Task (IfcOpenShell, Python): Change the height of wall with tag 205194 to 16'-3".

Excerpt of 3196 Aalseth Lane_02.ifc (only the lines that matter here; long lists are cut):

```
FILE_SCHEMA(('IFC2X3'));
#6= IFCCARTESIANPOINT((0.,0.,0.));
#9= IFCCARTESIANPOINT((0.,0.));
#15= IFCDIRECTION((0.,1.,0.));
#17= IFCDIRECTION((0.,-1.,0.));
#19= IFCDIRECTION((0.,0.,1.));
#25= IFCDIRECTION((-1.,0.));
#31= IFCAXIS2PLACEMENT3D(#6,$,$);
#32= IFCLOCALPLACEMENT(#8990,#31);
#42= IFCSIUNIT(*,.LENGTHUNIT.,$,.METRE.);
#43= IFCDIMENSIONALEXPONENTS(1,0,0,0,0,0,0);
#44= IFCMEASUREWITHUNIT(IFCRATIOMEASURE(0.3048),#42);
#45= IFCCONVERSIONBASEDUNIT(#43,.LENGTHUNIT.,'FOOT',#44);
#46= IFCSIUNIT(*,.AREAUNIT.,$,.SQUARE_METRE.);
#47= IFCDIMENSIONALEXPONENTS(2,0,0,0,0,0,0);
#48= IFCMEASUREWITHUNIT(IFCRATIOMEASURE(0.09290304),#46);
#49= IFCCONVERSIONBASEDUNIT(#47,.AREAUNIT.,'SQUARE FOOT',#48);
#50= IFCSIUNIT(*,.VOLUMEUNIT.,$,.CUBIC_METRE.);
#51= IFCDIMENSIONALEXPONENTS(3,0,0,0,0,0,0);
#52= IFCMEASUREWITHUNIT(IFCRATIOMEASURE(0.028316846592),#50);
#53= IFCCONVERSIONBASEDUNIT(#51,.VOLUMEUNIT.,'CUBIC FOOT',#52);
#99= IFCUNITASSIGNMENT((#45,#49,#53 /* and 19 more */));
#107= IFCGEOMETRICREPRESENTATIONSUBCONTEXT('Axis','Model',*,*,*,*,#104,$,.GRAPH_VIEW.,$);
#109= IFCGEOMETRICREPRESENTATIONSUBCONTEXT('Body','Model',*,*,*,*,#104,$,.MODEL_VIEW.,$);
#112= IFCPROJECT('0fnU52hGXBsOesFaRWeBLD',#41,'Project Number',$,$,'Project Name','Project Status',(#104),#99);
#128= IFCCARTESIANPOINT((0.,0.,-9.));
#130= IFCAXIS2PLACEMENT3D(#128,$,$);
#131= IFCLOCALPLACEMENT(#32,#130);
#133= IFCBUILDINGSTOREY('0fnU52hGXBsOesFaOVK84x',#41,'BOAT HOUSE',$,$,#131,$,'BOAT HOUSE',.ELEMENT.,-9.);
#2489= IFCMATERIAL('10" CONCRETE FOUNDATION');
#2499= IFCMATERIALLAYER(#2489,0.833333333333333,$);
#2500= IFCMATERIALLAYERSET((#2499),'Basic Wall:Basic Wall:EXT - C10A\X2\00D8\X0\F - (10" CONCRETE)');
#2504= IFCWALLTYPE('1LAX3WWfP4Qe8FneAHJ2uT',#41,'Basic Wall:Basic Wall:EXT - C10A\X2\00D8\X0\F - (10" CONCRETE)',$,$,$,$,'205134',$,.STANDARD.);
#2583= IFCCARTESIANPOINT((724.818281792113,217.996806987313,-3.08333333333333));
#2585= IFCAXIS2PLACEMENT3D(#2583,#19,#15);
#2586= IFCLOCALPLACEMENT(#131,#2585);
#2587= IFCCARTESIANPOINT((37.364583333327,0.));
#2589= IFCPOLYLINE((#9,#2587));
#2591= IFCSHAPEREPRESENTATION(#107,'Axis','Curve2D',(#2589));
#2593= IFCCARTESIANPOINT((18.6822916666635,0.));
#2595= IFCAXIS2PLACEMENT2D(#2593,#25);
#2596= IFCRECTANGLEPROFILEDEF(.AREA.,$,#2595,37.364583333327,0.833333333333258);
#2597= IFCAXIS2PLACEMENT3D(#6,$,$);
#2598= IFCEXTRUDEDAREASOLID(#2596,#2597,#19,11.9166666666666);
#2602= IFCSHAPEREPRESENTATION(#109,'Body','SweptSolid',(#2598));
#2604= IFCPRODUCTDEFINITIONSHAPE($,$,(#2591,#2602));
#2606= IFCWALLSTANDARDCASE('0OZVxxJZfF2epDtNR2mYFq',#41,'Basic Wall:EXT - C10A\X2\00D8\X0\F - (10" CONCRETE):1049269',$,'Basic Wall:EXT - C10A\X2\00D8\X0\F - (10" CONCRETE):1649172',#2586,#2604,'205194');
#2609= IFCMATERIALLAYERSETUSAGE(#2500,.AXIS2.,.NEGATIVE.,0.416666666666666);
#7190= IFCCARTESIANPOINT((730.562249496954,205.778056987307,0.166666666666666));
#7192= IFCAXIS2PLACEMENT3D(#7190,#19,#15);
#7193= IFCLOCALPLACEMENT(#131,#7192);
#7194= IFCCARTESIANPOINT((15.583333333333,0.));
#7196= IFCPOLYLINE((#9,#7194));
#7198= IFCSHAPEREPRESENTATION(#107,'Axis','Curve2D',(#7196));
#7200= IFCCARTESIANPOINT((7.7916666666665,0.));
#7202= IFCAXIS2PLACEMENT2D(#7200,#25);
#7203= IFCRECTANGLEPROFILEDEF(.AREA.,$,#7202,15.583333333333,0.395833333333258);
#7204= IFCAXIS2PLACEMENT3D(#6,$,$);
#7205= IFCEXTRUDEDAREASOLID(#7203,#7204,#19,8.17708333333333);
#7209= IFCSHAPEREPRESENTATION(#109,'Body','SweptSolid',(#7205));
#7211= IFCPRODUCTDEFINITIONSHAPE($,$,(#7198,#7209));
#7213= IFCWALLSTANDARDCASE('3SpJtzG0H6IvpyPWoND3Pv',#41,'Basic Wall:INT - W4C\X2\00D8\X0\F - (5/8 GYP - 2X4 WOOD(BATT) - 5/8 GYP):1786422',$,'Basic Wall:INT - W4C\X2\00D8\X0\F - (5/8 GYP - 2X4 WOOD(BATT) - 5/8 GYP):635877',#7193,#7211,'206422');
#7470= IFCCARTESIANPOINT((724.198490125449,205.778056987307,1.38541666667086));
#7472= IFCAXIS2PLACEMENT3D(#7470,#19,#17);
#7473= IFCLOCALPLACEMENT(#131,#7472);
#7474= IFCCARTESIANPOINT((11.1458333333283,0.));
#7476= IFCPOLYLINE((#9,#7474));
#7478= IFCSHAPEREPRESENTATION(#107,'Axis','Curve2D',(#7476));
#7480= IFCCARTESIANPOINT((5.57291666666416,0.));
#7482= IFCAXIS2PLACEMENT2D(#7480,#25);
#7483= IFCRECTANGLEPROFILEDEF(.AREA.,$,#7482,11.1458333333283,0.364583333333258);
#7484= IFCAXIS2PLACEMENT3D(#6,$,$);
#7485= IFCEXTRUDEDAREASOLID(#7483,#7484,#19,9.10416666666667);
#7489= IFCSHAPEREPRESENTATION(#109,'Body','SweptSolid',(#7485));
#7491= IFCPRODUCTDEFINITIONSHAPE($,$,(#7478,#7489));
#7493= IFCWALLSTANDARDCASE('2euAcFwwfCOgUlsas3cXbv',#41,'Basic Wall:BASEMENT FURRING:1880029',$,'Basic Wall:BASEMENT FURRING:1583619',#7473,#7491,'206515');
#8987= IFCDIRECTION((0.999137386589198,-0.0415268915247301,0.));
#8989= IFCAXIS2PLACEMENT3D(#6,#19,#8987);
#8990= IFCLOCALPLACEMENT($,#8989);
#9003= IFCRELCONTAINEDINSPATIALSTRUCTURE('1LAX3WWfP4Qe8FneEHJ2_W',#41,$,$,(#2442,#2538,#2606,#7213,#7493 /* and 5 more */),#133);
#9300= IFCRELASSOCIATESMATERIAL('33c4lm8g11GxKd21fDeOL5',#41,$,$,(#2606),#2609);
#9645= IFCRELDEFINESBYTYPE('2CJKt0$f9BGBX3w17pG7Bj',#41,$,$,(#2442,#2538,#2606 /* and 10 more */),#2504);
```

```python
import ifcopenshell
import ifcopenshell.geom
import ifcopenshell.util.representation
import ifcopenshell.util.shape
import ifcopenshell.util.unit

model = ifcopenshell.open("3196 Aalseth Lane_02.ifc")
unit_scale = ifcopenshell.util.unit.calculate_unit_scale(model)
settings = ifcopenshell.geom.settings()


def volume(element):
    """Net volume in cubic metres, openings subtracted."""
    shape = ifcopenshell.geom.create_shape(settings, element)
    return ifcopenshell.util.shape.get_volume(shape.geometry)


wall = model.by_id(2606)
before = volume(wall)

body = ifcopenshell.util.representation.get_representation(wall, "Model", "Body")
solid = body.Items[0]
old_height = solid.Depth
solid.Depth = 195 * 0.0254 / unit_scale
after = volume(wall)

print(f"height {old_height:g} -> {solid.Depth:g}, volume {before:.3f} -> {after:.3f} m3")

model.write("3196 Aalseth Lane_02_updated.ifc")
```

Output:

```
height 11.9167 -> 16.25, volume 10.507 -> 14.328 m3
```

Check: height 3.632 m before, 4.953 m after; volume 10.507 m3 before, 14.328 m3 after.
